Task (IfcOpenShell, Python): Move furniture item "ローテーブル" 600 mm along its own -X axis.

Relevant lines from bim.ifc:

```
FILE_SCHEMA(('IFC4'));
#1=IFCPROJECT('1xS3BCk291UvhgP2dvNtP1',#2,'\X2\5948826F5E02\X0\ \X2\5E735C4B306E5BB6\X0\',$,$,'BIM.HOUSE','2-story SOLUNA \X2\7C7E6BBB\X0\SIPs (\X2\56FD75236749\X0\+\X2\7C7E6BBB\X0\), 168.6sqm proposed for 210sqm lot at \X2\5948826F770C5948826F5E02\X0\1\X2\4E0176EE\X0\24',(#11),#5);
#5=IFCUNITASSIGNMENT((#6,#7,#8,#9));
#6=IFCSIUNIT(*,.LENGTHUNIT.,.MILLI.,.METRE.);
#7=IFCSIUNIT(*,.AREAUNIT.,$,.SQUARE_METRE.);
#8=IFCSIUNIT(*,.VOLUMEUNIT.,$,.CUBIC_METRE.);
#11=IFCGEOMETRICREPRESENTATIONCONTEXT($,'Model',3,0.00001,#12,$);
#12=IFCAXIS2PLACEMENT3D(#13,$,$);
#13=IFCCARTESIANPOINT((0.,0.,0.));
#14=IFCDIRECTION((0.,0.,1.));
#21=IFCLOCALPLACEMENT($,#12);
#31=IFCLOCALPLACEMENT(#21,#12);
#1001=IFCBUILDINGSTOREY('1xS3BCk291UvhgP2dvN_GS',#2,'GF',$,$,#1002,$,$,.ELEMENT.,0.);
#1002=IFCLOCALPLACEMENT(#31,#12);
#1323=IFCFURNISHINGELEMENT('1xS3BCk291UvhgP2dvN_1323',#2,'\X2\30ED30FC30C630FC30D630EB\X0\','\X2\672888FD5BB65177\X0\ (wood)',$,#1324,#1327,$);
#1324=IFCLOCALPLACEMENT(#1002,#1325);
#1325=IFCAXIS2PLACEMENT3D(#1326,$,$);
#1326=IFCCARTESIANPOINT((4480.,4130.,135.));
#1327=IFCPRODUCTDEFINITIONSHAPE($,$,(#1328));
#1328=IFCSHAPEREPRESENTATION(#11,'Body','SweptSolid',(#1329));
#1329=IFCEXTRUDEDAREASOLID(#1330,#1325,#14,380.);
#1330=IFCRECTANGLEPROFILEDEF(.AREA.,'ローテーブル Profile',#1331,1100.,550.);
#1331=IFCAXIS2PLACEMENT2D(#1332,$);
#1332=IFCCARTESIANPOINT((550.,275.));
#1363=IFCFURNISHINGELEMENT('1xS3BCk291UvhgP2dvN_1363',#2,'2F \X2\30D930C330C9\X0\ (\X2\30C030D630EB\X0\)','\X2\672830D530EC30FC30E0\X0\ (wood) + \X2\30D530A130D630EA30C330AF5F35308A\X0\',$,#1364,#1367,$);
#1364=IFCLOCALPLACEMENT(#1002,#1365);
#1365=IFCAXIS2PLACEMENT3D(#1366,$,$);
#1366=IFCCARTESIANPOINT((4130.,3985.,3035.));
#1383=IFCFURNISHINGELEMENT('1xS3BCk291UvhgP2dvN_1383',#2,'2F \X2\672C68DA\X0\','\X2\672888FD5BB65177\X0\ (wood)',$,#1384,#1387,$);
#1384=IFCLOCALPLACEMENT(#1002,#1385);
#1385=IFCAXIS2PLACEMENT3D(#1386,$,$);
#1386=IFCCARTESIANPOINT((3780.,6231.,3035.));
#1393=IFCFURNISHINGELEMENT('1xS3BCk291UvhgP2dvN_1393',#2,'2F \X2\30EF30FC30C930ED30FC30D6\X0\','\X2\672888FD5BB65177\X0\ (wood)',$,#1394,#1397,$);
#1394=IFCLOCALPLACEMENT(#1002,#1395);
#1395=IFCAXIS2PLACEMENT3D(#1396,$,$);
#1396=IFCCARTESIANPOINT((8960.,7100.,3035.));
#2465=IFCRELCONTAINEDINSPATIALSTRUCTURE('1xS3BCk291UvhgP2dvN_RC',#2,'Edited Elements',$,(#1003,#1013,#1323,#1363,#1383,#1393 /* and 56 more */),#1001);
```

```python
import ifcopenshell
import ifcopenshell.api.geometry
import ifcopenshell.util.placement
import ifcopenshell.util.unit

model = ifcopenshell.open("bim.ifc")
unit_scale = ifcopenshell.util.unit.calculate_unit_scale(model)

item = model.by_guid("1xS3BCk291UvhgP2dvN_1323")
matrix = ifcopenshell.util.placement.get_local_placement(item.ObjectPlacement)
matrix[:3, 3] -= matrix[:3, 0] * 0.6 / unit_scale
ifcopenshell.api.geometry.edit_object_placement(model, product=item, matrix=matrix, is_si=False)

print(ifcopenshell.util.placement.get_local_placement(item.ObjectPlacement).round(3) + 0.0)

model.write("bim_v2.ifc")
```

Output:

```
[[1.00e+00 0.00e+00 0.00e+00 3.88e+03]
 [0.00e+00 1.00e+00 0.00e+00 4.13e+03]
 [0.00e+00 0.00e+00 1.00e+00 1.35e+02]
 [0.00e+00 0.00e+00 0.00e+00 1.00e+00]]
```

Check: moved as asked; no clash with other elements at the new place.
